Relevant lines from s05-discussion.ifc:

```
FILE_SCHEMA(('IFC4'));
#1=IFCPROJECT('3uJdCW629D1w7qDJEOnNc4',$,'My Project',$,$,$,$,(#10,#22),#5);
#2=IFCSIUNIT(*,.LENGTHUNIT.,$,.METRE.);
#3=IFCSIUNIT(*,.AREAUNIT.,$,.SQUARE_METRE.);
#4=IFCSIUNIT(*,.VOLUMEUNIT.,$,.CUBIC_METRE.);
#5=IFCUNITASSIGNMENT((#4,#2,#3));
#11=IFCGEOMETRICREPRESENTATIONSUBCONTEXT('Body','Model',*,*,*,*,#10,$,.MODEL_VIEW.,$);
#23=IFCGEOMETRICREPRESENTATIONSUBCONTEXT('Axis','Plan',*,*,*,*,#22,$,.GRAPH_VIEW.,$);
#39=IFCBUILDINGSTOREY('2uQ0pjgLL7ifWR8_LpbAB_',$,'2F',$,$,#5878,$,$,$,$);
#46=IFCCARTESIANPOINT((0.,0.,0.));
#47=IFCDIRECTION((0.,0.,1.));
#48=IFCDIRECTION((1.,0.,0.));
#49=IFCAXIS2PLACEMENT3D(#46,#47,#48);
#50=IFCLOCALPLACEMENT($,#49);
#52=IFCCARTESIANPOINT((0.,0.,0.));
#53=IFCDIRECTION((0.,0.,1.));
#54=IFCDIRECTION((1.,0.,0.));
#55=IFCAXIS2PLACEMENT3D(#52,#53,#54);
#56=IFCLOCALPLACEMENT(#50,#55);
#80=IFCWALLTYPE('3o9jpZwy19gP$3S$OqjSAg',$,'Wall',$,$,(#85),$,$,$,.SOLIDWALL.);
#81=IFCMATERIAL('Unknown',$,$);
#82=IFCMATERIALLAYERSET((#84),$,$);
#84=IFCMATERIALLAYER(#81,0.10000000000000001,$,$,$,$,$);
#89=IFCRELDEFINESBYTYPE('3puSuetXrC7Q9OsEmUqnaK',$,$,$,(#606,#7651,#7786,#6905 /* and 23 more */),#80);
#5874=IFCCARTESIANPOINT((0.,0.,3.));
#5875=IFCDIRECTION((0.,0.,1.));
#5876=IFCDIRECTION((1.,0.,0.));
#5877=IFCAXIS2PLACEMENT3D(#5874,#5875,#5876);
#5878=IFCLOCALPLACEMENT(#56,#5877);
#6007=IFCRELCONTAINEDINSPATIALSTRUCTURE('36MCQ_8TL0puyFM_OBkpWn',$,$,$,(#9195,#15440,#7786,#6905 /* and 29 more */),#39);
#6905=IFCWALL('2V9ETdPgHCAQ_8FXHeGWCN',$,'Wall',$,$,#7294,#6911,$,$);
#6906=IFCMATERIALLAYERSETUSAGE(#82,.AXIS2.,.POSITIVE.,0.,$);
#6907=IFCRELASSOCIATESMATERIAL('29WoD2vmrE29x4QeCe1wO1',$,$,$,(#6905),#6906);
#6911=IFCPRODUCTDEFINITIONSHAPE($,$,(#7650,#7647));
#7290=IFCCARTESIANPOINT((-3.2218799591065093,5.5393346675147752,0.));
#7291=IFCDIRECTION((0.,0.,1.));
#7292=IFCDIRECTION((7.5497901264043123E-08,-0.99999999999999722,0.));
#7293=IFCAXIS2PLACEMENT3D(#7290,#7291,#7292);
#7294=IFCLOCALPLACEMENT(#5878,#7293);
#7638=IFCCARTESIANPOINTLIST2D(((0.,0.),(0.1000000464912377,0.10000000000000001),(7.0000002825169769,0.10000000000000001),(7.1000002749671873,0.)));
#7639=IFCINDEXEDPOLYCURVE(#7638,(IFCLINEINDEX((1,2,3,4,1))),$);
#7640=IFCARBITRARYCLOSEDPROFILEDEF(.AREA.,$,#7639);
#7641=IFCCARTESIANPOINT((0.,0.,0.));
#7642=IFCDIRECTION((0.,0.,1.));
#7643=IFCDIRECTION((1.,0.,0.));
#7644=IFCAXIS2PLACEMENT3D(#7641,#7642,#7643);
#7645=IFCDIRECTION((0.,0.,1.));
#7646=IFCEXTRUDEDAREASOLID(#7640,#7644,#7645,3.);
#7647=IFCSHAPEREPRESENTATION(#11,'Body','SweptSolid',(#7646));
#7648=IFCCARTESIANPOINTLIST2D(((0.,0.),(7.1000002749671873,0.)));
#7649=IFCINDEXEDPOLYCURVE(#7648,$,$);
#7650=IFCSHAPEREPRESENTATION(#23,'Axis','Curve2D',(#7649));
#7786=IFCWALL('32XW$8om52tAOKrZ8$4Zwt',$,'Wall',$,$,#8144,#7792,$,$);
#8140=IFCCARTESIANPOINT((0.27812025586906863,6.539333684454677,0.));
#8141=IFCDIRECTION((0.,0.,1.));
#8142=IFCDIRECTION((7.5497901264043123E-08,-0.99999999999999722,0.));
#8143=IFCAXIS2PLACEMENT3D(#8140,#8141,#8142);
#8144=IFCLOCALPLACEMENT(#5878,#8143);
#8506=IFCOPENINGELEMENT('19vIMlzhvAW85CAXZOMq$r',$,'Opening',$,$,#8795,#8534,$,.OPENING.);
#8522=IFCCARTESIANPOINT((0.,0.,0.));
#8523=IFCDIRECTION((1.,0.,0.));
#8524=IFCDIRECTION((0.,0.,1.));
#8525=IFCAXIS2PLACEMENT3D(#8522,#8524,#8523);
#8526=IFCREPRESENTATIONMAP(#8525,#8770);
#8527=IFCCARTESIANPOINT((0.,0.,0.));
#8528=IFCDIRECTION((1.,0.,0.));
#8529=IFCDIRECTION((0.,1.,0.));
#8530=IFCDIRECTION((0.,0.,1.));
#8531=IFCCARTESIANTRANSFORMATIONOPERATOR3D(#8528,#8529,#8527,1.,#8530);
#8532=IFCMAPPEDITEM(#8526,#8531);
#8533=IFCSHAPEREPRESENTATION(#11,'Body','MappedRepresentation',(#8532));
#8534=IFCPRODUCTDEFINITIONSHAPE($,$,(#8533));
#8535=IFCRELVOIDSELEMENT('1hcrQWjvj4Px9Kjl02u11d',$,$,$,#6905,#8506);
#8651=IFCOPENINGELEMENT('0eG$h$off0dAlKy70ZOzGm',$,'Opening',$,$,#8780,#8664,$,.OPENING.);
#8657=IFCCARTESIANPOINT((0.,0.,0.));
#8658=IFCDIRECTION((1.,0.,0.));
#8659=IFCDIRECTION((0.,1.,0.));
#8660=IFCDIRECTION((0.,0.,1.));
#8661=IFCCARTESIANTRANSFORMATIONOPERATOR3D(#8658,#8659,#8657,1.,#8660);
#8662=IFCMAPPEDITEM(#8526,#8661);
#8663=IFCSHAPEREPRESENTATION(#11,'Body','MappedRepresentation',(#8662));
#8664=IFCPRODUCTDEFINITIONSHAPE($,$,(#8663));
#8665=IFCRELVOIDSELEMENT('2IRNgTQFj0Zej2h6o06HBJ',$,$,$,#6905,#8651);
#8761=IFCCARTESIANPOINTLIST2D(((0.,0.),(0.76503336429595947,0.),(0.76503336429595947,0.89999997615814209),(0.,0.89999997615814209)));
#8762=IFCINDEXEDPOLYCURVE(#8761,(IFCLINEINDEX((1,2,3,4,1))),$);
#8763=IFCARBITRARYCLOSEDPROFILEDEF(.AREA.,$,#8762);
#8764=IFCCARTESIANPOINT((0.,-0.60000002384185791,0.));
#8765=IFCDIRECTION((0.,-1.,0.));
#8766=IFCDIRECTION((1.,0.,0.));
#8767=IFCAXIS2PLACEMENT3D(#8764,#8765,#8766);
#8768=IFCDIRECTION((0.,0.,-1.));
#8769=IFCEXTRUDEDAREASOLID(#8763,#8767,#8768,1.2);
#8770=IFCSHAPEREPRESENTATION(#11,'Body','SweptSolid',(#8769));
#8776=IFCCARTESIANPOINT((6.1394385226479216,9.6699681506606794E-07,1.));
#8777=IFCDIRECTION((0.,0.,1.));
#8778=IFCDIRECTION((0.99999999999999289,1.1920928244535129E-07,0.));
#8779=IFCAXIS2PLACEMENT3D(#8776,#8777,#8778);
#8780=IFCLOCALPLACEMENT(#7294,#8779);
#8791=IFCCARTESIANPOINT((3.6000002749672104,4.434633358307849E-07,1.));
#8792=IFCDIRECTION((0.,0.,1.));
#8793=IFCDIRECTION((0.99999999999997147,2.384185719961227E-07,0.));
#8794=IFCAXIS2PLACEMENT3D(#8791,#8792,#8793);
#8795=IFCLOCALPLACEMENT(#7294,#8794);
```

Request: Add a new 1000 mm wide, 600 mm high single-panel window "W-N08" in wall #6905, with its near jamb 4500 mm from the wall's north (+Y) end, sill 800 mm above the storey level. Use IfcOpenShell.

```python
import numpy as np
import ifcopenshell
import ifcopenshell.api.feature
import ifcopenshell.api.geometry
import ifcopenshell.api.root
import ifcopenshell.api.spatial
import ifcopenshell.geom
import ifcopenshell.util.element
import ifcopenshell.util.placement
import ifcopenshell.util.representation
import ifcopenshell.util.shape
import ifcopenshell.util.unit

model = ifcopenshell.open("s05-discussion.ifc")
unit_scale = ifcopenshell.util.unit.calculate_unit_scale(model)
settings = ifcopenshell.geom.settings()


def volume(element):
    """Net volume in cubic metres, openings subtracted."""
    shape = ifcopenshell.geom.create_shape(settings, element)
    return ifcopenshell.util.shape.get_volume(shape.geometry)


wall = model.by_guid("2V9ETdPgHCAQ_8FXHeGWCN")
storey = ifcopenshell.util.element.get_container(wall, ifc_class="IfcBuildingStorey")
context = ifcopenshell.util.representation.get_context(model, "Model", "Body", "MODEL_VIEW")
before = volume(wall)

width, height, from_end, sill = 1, 0.6, 4.5, 0.8  # metres

# The wall runs along its own X axis, and the end named is its -X end.
wall_shape = ifcopenshell.geom.create_shape(settings, wall)
x, y, z = ifcopenshell.util.shape.get_vertices(wall_shape.geometry).T
start = x.min() + from_end
face, thickness = float(y.min()), float(y.max() - y.min())
wall_matrix = ifcopenshell.util.placement.get_local_placement(wall.ObjectPlacement)
level = ifcopenshell.util.placement.get_local_placement(storey.ObjectPlacement)[2, 3]


def in_wall(x, y):
    """Placement at x, y metres in the wall's axes, at sill height."""
    matrix = wall_matrix.copy()
    matrix[:, 3] = wall_matrix @ np.array([x / unit_scale, y / unit_scale, 0.0, 1.0])
    matrix[2, 3] = level + sill / unit_scale
    return matrix


# Opening: a box that overshoots both wall faces by 50 mm.
opening = ifcopenshell.api.root.create_entity(model, ifc_class="IfcOpeningElement", predefined_type="OPENING")
box = ifcopenshell.api.geometry.add_wall_representation(
    model, context=context, length=width, height=height, thickness=thickness + 0.1
)
ifcopenshell.api.geometry.assign_representation(model, product=opening, representation=box)
ifcopenshell.api.geometry.edit_object_placement(model, product=opening, matrix=in_wall(start, face - 0.05), is_si=False)
ifcopenshell.api.feature.add_feature(model, feature=opening, element=wall)

window = ifcopenshell.api.root.create_entity(model, ifc_class="IfcWindow", name="W-N08", predefined_type="WINDOW")
window.OverallWidth, window.OverallHeight = width / unit_scale, height / unit_scale
window.PartitioningType = "SINGLE_PANEL"
body = ifcopenshell.api.geometry.add_window_representation(
    model,
    context=context,
    overall_width=window.OverallWidth,
    overall_height=window.OverallHeight,
    partition_type="SINGLE_PANEL",
)
ifcopenshell.api.geometry.assign_representation(model, product=window, representation=body)
ifcopenshell.api.spatial.assign_container(model, products=[window], relating_structure=storey)
ifcopenshell.api.feature.add_filling(model, opening=opening, element=window)

# Centre the window in the wall's thickness.
ifcopenshell.api.geometry.edit_object_placement(model, product=window, matrix=in_wall(start, face), is_si=False)
window_shape = ifcopenshell.geom.create_shape(settings, window)
depth = ifcopenshell.util.shape.get_vertices(window_shape.geometry)[:, 1]
offset = face + thickness / 2 - (depth.min() + depth.max()) / 2
ifcopenshell.api.geometry.edit_object_placement(model, product=window, matrix=in_wall(start, offset), is_si=False)

after = volume(wall)

print(f"wall volume {before:.3f} -> {after:.3f} m3")

model.write("s05-discussion-out.ifc")
```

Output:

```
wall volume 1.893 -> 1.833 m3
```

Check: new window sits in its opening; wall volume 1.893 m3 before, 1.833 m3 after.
